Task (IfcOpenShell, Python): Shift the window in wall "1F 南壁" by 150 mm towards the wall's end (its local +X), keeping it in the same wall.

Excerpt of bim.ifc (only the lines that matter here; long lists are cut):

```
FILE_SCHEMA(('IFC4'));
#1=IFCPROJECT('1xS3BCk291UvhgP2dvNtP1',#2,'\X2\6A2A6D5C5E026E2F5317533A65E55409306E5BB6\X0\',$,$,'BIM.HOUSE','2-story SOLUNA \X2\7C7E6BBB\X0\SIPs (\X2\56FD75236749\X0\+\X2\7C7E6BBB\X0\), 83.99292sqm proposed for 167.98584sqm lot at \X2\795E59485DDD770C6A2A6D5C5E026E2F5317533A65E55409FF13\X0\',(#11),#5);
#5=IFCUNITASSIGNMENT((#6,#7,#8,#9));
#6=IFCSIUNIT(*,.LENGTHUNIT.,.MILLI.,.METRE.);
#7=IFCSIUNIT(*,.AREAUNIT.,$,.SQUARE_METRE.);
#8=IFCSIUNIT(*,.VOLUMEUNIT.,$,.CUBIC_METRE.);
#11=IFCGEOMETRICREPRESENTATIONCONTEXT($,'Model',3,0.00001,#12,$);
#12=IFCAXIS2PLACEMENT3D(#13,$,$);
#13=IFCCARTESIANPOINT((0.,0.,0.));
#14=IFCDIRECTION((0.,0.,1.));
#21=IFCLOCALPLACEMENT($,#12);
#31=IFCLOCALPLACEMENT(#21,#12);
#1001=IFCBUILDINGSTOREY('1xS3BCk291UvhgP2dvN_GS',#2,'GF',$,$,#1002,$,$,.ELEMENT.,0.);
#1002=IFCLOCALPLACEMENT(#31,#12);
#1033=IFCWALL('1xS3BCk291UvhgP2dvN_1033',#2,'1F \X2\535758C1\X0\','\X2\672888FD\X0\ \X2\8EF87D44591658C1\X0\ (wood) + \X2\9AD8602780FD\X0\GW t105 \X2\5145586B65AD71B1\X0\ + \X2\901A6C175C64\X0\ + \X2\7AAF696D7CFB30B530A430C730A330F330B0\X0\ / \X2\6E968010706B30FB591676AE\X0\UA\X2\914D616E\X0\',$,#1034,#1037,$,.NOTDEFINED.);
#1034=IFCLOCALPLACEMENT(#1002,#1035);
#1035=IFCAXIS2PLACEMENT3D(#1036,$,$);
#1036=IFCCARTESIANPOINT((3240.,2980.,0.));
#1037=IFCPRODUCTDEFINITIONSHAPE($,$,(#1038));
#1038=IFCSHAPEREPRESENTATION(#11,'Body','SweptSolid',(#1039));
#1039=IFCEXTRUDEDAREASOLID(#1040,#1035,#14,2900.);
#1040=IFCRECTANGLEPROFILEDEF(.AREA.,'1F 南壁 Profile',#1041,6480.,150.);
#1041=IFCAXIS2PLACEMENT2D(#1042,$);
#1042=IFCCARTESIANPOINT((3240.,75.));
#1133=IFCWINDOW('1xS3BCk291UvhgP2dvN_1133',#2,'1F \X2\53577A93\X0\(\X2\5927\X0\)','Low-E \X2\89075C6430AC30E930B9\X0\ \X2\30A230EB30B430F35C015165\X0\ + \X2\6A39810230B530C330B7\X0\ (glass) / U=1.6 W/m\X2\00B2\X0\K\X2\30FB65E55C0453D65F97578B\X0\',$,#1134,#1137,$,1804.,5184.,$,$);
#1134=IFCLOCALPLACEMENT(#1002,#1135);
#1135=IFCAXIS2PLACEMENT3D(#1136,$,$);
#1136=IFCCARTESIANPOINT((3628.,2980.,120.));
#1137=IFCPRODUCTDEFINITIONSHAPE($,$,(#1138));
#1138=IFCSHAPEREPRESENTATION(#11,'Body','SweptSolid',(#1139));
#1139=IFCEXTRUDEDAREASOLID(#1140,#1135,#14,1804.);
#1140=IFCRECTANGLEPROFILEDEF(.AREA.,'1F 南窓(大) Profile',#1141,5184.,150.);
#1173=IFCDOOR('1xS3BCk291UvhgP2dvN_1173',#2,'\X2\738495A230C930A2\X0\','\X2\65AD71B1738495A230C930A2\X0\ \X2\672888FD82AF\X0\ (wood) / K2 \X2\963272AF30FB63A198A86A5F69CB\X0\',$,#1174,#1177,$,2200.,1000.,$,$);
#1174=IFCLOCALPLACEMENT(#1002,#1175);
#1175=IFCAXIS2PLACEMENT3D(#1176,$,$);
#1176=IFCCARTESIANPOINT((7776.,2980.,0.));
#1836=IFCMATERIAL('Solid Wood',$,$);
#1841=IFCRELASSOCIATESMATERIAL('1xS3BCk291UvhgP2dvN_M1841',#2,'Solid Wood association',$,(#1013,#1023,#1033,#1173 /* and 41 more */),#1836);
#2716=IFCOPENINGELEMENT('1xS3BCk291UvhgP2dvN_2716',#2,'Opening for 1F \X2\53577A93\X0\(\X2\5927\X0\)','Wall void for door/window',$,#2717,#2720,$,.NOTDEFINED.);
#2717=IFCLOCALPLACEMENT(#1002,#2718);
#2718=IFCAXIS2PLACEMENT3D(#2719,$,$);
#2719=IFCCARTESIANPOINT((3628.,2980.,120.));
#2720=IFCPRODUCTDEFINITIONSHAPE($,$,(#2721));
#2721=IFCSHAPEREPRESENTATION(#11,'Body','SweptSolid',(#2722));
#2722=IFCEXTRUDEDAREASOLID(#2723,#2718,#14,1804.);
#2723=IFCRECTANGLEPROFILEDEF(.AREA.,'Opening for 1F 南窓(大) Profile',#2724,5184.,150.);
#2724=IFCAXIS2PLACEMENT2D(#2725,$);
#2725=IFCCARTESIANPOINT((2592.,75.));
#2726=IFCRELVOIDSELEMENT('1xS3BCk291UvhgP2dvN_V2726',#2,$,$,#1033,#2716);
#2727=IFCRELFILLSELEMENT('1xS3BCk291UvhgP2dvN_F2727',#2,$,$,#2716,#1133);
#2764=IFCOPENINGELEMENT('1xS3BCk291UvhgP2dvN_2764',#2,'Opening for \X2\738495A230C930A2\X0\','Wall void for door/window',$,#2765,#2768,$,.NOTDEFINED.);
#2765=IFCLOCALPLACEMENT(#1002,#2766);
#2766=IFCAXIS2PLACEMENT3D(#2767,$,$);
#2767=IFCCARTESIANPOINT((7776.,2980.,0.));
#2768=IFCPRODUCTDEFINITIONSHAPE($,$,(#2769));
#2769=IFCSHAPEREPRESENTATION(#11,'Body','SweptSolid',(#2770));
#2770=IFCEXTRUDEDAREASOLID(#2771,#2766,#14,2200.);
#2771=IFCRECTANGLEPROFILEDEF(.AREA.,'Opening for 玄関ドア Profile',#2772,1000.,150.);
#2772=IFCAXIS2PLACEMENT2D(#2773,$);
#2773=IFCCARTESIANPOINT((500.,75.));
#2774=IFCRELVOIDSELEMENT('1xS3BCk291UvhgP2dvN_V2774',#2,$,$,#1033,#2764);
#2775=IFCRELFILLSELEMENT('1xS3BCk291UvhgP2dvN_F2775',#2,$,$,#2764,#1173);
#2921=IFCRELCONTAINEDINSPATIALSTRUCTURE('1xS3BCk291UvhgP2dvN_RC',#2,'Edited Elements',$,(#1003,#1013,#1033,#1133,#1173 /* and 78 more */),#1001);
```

```python
import ifcopenshell
import ifcopenshell.api.geometry
import ifcopenshell.util.placement
import ifcopenshell.util.unit

model = ifcopenshell.open("bim.ifc")
unit_scale = ifcopenshell.util.unit.calculate_unit_scale(model)

window = model.by_guid("1xS3BCk291UvhgP2dvN_1133")
opening = window.FillsVoids[0].RelatingOpeningElement
wall = opening.VoidsElements[0].RelatingBuildingElement

wall_matrix = ifcopenshell.util.placement.get_local_placement(wall.ObjectPlacement)
shift = wall_matrix[:3, 0] * 0.15 / unit_scale
before = ifcopenshell.util.placement.get_local_placement(window.ObjectPlacement)[:3, 3].copy()

# The window is not placed relative to its opening, so move both.
for product in (opening, window):
    matrix = ifcopenshell.util.placement.get_local_placement(product.ObjectPlacement)
    matrix[:3, 3] += shift
    ifcopenshell.api.geometry.edit_object_placement(model, product=product, matrix=matrix, is_si=False)

after = ifcopenshell.util.placement.get_local_placement(window.ObjectPlacement)[:3, 3]
print("window moved by", (after - before).round(3) + 0.0)

model.write("bim_updated.ifc")
```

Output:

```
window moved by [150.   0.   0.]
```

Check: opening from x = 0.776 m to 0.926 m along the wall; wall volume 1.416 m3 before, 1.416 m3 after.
